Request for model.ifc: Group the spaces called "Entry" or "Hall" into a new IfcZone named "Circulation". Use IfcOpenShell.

First a look at what the model holds.

```python
import ifcopenshell

model = ifcopenshell.open("model.ifc")
print(model.schema)
seen = {}
for space in model.by_type("IfcSpace"):
    seen[space.LongName] = seen.get(space.LongName, 0) + 1
for name, count in sorted(seen.items(), key=str):
    print(count, "x", name)
print("zones:", [z.Name for z in model.by_type("IfcZone")][:20])
```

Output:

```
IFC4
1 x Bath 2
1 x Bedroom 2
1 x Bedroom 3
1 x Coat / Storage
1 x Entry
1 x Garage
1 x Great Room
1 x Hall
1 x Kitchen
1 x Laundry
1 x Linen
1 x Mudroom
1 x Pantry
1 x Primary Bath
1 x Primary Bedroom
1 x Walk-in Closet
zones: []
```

```python
import ifcopenshell
import ifcopenshell.api.group
import ifcopenshell.api.root

model = ifcopenshell.open("model.ifc")

names = {"Entry", "Hall"}
spaces = [s for s in model.by_type("IfcSpace") if s.LongName in names]

zone = ifcopenshell.api.root.create_entity(model, ifc_class="IfcZone", name="Circulation")
ifcopenshell.api.group.assign_group(model, products=spaces, group=zone)
print(len(spaces), "spaces in", zone.Name)

model.write("model_edited.ifc")
```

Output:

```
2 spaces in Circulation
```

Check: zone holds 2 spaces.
